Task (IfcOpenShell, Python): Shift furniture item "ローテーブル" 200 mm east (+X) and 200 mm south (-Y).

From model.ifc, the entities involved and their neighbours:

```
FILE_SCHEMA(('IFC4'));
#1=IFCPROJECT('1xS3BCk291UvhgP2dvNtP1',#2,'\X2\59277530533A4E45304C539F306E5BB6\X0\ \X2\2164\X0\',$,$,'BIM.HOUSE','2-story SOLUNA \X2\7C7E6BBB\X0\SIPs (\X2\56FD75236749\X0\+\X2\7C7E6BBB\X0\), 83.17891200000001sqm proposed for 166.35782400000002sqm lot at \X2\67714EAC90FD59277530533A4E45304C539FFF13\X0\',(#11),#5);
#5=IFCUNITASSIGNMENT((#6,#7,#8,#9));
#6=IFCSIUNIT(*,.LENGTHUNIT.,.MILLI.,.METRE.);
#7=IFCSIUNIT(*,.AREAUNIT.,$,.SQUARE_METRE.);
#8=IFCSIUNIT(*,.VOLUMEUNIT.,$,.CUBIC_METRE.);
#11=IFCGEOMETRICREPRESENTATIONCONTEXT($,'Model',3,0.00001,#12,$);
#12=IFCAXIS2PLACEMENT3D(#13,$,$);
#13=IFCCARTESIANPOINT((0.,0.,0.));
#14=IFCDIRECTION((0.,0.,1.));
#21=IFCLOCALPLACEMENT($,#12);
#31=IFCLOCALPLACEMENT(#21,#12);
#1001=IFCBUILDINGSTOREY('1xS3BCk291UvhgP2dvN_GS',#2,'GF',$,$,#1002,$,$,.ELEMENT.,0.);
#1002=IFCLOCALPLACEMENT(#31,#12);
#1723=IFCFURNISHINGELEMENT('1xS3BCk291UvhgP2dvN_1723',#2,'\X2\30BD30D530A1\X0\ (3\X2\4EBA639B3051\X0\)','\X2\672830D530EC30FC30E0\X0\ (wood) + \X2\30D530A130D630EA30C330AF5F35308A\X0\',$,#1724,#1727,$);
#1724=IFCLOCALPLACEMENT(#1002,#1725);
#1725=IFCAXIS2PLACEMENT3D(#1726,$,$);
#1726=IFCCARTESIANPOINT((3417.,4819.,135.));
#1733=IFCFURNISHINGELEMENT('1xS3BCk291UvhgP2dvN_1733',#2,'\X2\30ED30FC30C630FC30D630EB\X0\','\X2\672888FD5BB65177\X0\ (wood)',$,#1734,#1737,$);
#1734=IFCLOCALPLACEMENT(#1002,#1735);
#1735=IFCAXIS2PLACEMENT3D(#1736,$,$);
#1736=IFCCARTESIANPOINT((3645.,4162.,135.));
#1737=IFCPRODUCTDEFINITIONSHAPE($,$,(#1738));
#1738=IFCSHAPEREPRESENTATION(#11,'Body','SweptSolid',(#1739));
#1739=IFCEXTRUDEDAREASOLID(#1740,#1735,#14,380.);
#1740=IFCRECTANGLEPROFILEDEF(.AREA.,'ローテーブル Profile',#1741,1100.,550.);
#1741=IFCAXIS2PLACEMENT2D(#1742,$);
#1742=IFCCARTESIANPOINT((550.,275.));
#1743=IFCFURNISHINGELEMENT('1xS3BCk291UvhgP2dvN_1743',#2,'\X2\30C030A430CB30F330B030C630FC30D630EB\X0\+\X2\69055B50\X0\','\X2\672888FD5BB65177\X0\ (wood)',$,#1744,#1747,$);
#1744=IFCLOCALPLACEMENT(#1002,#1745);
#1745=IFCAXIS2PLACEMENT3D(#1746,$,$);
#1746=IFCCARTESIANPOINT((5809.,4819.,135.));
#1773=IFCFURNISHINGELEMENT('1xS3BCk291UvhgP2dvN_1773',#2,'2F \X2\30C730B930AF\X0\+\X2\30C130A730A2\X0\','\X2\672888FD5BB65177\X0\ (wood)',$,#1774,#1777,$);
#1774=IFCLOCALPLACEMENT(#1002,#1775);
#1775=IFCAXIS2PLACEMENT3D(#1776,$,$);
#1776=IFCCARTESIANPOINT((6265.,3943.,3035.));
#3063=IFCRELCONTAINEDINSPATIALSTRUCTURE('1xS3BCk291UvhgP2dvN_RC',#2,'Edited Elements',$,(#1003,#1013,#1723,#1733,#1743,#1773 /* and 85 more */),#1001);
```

```python
import ifcopenshell
import ifcopenshell.api.geometry
import ifcopenshell.util.placement
import ifcopenshell.util.unit

model = ifcopenshell.open("model.ifc")
unit_scale = ifcopenshell.util.unit.calculate_unit_scale(model)

item = model.by_guid("1xS3BCk291UvhgP2dvN_1733")
matrix = ifcopenshell.util.placement.get_local_placement(item.ObjectPlacement)
matrix[0, 3] += 0.2 / unit_scale
matrix[1, 3] -= 0.2 / unit_scale
ifcopenshell.api.geometry.edit_object_placement(model, product=item, matrix=matrix, is_si=False)

print(ifcopenshell.util.placement.get_local_placement(item.ObjectPlacement).round(3) + 0.0)

model.write("model-out.ifc")
```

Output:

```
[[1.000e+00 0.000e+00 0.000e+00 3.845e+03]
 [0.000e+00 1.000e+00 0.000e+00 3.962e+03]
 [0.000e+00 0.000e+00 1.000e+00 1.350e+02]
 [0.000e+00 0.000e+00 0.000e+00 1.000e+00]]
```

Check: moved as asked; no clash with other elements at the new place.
